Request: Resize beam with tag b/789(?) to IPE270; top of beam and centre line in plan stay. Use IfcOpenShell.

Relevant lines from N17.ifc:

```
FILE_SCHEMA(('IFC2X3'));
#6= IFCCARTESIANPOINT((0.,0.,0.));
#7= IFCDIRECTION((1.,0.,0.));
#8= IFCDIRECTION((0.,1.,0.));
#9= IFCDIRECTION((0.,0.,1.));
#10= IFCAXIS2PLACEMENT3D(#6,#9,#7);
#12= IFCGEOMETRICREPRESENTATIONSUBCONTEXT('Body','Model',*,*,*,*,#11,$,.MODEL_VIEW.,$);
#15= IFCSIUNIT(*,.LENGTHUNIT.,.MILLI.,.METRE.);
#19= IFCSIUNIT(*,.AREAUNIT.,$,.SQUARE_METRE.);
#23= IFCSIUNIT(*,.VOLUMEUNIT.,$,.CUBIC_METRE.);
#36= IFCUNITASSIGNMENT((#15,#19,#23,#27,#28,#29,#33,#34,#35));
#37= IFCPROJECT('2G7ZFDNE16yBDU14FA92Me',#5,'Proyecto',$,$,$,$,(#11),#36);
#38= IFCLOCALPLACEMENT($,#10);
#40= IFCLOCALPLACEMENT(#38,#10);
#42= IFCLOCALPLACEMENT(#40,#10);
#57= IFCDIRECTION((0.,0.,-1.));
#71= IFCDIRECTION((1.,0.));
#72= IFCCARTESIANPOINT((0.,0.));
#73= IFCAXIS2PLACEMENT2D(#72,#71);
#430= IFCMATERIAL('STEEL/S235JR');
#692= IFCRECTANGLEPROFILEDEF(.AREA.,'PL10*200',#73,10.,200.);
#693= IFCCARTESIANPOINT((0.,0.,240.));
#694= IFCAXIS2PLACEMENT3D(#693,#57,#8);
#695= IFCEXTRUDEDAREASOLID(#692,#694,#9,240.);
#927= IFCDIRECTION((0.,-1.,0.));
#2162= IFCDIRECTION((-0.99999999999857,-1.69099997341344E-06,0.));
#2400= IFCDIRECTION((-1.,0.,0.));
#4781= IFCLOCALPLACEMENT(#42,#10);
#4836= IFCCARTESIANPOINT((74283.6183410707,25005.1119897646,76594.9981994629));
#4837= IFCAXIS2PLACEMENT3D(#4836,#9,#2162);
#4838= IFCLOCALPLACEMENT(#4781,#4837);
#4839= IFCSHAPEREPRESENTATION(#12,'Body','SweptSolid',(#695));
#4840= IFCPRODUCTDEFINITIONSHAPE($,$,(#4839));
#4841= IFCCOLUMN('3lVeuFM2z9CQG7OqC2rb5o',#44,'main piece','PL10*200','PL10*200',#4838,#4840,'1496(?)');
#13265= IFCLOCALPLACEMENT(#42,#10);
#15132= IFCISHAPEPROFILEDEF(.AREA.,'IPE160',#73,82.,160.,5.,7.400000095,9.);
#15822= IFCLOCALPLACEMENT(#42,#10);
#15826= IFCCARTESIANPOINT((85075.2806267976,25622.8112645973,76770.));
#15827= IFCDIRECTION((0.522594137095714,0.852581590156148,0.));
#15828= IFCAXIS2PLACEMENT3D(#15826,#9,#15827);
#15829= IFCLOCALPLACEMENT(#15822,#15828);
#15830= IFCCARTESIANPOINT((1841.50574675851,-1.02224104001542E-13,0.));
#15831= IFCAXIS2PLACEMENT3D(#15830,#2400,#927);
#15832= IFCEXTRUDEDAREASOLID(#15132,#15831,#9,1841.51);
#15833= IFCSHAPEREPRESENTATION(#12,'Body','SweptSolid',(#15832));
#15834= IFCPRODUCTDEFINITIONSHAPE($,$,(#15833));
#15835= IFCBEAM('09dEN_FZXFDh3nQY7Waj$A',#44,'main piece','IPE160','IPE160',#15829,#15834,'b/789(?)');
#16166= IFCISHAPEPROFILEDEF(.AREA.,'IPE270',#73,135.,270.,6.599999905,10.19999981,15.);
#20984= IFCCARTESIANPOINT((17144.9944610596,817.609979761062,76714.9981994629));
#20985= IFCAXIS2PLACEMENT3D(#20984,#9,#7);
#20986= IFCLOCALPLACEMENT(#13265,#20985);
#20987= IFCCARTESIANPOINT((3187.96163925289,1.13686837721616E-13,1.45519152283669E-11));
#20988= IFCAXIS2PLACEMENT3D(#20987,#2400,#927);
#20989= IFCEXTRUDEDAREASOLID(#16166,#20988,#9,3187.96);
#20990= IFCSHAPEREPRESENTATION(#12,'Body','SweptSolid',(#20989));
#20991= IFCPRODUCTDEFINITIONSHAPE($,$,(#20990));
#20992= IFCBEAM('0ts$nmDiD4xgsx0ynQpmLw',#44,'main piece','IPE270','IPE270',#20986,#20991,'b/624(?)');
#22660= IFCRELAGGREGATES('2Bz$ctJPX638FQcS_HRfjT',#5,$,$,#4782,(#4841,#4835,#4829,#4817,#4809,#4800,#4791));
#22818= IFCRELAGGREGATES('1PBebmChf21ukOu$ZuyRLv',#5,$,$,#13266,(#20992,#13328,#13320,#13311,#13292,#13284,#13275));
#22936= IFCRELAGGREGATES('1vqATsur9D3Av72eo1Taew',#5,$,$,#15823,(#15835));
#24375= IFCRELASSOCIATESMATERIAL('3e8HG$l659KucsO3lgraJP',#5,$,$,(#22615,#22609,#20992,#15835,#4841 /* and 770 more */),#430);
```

```python
import ifcopenshell
import ifcopenshell.util.element
import ifcopenshell.util.representation

model = ifcopenshell.open("N17.ifc")

member = model.by_guid("09dEN_FZXFDh3nQY7Waj$A")
source = next(p for p in model.by_type("IfcIShapeProfileDef") if p.ProfileName == "IPE270")

body = ifcopenshell.util.representation.get_representation(member, "Model", "Body")
solid = body.Items[0]
old_profile = solid.SweptArea

# Copy the section's sizes but keep this member's own profile position.
profile = ifcopenshell.util.element.copy(model, source)
# Profiles are centred, so shift by half the change in depth to hold the top.
shift = (old_profile.OverallDepth - profile.OverallDepth) / 2
x, y = old_profile.Position.Location.Coordinates
up = (0.0, 1.0)  # upwards, in the solid's own plane
location = model.createIfcCartesianPoint((x + up[0] * shift, y + up[1] * shift))
profile.Position = model.createIfcAxis2Placement2D(location, old_profile.Position.RefDirection)
solid.SweptArea = profile
if not model.get_total_inverses(old_profile):
    ifcopenshell.util.element.remove_deep2(model, old_profile)
member.Description = member.Description.replace("IPE160", "IPE270")
member.ObjectType = member.ObjectType.replace("IPE160", "IPE270")

print(solid.SweptArea)

model.write("N17-out.ifc")
```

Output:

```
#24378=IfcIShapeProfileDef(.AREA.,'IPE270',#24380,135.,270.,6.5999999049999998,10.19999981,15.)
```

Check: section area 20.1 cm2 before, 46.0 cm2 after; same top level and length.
